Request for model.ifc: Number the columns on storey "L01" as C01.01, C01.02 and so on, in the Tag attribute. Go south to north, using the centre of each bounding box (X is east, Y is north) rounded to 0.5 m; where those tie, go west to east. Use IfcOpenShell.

First a look at what the model holds.

```python
import ifcopenshell
import ifcopenshell.util.element
import ifcopenshell.util.placement

model = ifcopenshell.open("model.ifc")
print(model.schema)
storey = next(s for s in model.by_type("IfcBuildingStorey") if s.Name == "L01")
columns = [e for e in ifcopenshell.util.element.get_decomposition(storey) if e.is_a("IfcColumn")]
for e in sorted(columns, key=lambda e: e.id()):
    origin = ifcopenshell.util.placement.get_local_placement(e.ObjectPlacement)[:3, 3]
    print(e.id(), e.Tag, e.Name, origin.round(2) + 0.0, sep=" | ")
```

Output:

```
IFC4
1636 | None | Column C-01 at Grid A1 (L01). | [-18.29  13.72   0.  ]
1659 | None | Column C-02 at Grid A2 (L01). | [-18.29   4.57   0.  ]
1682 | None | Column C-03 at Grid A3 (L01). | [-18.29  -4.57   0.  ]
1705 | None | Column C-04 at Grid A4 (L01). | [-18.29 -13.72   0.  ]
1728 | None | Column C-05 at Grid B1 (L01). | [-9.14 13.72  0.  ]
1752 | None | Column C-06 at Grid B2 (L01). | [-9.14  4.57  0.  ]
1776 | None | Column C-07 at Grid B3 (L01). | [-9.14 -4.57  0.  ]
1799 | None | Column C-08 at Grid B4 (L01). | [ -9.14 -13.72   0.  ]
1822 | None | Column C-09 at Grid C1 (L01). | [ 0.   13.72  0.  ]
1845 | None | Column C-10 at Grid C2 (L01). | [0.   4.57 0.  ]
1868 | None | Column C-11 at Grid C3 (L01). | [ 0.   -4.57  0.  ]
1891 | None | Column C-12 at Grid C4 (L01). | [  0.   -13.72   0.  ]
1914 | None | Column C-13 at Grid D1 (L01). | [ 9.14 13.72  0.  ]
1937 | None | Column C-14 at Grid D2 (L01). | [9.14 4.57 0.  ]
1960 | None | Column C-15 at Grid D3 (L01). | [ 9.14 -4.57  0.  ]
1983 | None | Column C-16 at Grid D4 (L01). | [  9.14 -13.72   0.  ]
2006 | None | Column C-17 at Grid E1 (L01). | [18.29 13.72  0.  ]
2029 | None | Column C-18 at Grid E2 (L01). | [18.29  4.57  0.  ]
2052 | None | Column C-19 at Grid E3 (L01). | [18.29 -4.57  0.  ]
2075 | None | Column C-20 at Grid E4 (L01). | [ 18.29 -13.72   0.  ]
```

```python
import ifcopenshell
import ifcopenshell.geom
import ifcopenshell.util.element
import ifcopenshell.util.shape

model = ifcopenshell.open("model.ifc")
settings = ifcopenshell.geom.settings()
settings.set("use-world-coords", True)


def centre(element):
    shape = ifcopenshell.geom.create_shape(settings, element)
    return ifcopenshell.util.shape.get_bbox_centroid(shape.geometry)


storey = next(s for s in model.by_type("IfcBuildingStorey") if s.Name == "L01")
columns = [e for e in ifcopenshell.util.element.get_decomposition(storey) if e.is_a("IfcColumn")]

# Insertion points can sit at a corner or the storey origin, so sort by the geometry (in metres).
centres = {e: centre(e) for e in columns}
columns.sort(key=lambda e: (round(centres[e][1] / 0.5), centres[e][0]))

for i, e in enumerate(columns, start=1):
    number = f"C01.{i:02d}"
    e.Tag = number
    print(e.id(), number)

model.write("model-out.ifc")
```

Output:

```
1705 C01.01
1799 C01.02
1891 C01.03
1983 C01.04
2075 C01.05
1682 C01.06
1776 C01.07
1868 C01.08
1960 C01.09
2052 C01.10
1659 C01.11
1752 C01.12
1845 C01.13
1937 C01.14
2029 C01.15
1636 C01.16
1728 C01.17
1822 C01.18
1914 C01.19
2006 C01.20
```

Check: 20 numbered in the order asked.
